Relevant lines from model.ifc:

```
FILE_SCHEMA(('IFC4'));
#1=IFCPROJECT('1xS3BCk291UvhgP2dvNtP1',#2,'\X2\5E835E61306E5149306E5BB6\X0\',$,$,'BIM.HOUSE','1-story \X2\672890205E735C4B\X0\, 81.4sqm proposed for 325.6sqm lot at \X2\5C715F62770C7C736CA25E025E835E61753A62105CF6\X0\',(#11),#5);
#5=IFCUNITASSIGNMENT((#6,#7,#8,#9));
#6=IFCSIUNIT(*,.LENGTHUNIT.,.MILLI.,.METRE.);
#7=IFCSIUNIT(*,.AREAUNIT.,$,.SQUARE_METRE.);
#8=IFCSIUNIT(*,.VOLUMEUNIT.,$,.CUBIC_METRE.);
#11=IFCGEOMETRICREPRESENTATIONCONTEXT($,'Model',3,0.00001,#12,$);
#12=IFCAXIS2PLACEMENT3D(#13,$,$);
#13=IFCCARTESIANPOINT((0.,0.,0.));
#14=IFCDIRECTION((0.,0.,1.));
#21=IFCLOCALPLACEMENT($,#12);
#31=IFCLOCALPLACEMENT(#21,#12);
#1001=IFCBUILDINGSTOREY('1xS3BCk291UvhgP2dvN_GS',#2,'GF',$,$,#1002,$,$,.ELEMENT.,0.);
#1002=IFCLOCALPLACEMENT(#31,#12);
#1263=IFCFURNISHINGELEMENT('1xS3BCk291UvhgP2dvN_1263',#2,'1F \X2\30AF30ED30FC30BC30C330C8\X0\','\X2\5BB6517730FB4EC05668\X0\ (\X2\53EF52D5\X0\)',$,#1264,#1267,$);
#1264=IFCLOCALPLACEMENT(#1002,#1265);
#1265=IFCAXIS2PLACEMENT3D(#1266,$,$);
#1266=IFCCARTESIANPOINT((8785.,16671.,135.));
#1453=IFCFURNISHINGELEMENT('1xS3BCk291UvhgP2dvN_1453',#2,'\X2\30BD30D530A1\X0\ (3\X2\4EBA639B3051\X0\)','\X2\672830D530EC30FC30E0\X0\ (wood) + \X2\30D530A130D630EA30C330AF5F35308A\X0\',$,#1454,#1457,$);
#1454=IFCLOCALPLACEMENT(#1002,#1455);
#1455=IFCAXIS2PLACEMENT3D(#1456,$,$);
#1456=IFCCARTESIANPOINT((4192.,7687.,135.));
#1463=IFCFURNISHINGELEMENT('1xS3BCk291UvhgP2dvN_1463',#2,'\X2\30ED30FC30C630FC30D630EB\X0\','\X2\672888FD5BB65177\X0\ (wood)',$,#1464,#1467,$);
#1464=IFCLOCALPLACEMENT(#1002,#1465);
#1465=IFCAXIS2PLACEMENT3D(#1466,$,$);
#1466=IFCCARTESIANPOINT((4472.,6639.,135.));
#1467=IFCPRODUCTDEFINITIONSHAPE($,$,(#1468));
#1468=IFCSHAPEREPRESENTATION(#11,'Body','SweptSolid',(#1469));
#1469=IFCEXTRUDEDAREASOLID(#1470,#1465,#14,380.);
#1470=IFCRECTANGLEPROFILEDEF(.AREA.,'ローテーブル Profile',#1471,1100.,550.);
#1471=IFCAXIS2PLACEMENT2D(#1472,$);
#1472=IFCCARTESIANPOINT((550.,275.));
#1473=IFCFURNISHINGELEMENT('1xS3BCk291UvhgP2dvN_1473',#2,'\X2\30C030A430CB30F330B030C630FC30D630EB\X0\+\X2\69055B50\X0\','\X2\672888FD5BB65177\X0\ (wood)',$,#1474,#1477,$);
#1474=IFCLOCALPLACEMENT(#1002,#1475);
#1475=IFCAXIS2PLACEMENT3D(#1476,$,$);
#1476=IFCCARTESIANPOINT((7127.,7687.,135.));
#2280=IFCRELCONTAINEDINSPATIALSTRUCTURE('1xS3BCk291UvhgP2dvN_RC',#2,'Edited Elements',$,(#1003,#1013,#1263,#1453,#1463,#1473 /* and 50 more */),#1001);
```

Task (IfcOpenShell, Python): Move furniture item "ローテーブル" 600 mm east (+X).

```python
import ifcopenshell
import ifcopenshell.api.geometry
import ifcopenshell.util.placement

model = ifcopenshell.open("model.ifc")

item = model.by_guid("1xS3BCk291UvhgP2dvN_1463")
matrix = ifcopenshell.util.placement.get_local_placement(item.ObjectPlacement)
matrix[0, 3] += 600.0
ifcopenshell.api.geometry.edit_object_placement(model, product=item, matrix=matrix, is_si=False)

print(ifcopenshell.util.placement.get_local_placement(item.ObjectPlacement).round(3) + 0.0)

model.write("model-out.ifc")
```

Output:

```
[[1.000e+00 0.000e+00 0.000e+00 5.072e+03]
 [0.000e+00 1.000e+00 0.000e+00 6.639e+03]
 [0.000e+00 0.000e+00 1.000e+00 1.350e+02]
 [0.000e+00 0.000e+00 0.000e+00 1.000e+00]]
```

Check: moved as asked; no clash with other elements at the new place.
